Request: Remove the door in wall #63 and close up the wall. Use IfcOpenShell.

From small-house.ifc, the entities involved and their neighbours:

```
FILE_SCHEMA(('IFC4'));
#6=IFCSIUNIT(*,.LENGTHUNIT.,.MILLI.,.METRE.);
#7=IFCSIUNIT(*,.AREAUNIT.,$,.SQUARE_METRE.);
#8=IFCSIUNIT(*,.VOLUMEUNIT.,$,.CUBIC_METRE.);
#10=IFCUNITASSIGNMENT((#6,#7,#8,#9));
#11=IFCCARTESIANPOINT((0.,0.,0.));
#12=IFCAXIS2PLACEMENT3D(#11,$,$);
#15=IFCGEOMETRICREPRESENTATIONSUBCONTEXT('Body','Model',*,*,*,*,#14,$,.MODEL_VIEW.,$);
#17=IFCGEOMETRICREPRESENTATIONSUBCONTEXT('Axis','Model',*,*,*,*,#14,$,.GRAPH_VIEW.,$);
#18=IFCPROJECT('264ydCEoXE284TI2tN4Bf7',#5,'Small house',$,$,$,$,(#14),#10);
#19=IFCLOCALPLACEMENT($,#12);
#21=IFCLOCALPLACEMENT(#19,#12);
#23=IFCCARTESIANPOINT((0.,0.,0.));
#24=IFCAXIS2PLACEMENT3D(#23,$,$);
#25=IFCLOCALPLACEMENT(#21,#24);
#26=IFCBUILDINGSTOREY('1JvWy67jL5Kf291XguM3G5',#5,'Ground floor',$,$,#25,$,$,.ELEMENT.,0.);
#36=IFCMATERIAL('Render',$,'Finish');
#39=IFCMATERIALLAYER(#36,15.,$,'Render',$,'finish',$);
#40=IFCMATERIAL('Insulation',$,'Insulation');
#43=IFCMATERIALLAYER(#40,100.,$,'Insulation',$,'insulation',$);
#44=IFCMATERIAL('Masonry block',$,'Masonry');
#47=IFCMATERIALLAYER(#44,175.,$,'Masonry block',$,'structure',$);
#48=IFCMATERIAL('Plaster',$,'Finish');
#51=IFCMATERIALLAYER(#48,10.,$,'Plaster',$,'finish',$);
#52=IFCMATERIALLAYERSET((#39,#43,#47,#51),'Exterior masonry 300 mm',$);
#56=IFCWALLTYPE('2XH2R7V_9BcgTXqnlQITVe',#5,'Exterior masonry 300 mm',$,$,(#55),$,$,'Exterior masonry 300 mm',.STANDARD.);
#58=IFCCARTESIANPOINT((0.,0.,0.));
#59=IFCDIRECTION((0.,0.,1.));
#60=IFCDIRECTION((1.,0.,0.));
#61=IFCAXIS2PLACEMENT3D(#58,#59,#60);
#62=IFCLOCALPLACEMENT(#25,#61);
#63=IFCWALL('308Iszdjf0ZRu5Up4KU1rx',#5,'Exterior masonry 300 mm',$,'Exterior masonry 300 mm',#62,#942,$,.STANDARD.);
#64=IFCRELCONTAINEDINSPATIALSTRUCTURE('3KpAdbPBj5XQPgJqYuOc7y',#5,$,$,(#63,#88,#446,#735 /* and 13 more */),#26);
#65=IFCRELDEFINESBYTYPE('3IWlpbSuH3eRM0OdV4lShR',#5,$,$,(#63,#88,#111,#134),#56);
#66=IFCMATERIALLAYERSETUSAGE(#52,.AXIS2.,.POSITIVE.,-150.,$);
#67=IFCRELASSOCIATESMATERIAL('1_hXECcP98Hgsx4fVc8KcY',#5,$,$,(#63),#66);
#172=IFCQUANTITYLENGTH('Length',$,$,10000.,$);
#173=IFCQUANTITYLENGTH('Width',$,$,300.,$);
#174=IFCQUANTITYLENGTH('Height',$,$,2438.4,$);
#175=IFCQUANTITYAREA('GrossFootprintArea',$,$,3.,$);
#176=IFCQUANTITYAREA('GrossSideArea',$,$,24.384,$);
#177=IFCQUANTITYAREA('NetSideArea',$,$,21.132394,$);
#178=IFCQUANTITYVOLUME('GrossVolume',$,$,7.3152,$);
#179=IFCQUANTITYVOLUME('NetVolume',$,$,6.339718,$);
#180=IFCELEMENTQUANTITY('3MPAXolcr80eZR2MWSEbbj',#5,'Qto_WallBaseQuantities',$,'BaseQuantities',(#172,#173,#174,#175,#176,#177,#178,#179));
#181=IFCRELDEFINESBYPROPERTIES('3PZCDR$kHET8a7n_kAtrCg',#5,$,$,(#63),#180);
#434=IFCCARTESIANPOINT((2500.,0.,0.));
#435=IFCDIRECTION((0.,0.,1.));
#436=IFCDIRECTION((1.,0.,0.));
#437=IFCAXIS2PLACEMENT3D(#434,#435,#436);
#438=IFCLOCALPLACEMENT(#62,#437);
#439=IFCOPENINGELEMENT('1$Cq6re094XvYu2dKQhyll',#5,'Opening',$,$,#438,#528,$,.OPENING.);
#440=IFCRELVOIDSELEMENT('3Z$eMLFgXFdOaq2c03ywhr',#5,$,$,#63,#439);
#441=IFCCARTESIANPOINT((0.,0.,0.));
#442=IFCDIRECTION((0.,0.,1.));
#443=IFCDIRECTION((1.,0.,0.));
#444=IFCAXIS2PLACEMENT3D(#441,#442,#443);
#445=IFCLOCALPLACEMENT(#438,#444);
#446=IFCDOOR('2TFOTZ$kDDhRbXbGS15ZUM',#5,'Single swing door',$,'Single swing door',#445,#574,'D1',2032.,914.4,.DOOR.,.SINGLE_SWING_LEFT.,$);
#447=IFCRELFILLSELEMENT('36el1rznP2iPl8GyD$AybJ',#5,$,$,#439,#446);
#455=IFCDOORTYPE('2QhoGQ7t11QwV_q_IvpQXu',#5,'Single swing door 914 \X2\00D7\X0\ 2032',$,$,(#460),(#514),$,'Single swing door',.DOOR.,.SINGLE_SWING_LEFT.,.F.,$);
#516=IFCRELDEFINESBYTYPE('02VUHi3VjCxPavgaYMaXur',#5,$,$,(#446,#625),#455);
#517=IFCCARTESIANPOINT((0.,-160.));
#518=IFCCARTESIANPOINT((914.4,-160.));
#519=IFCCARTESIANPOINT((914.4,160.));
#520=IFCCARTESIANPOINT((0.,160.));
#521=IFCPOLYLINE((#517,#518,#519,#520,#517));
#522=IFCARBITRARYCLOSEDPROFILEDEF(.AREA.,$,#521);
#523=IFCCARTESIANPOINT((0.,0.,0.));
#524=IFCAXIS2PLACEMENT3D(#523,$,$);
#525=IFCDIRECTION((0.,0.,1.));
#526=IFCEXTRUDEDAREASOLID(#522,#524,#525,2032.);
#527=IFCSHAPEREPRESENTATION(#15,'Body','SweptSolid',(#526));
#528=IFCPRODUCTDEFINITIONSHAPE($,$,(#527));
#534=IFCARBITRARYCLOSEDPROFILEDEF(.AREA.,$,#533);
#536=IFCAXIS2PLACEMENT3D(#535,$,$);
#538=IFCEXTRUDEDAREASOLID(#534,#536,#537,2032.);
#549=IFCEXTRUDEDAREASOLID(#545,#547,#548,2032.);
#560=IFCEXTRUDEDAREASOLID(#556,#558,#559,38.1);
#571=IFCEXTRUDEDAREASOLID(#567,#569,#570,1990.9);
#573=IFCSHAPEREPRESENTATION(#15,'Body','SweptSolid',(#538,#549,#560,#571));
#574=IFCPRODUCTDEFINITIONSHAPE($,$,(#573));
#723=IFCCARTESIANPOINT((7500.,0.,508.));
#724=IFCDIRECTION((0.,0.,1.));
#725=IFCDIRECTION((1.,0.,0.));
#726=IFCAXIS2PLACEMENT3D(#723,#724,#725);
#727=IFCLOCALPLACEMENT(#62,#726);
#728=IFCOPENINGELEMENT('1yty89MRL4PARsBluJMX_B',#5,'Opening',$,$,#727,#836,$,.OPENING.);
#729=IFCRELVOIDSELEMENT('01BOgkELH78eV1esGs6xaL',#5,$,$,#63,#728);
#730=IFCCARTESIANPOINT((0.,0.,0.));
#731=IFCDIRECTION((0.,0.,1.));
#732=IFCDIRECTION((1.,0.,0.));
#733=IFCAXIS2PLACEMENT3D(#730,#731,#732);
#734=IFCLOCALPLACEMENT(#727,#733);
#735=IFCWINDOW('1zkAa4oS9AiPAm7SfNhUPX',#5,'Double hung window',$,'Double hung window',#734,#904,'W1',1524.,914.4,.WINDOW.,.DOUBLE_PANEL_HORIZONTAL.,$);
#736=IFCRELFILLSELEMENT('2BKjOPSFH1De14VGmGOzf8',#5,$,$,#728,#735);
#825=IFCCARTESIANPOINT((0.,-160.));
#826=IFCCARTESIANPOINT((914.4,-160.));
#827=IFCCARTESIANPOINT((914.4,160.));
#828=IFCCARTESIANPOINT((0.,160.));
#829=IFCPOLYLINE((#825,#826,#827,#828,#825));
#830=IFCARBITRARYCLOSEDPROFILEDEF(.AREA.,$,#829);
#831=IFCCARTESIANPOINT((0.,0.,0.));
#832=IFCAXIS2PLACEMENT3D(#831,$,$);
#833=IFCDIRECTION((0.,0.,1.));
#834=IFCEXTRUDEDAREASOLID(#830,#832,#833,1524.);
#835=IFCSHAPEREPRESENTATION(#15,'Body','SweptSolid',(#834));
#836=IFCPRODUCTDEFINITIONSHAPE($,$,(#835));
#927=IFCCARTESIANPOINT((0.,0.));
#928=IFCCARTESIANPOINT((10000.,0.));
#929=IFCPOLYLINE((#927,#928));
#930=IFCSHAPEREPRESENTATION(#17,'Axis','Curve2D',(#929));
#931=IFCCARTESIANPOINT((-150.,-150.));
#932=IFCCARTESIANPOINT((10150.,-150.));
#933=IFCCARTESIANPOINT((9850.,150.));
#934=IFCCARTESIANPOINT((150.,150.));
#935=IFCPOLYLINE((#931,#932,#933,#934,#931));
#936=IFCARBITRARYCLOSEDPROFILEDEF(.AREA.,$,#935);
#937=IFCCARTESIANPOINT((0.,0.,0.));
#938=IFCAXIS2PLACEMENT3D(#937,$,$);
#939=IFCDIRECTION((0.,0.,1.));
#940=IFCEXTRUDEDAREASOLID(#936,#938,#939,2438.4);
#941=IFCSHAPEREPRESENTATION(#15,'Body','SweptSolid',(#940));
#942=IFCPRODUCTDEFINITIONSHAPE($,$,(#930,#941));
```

```python
import ifcopenshell
import ifcopenshell.api.feature
import ifcopenshell.api.pset
import ifcopenshell.api.root
import ifcopenshell.geom
import ifcopenshell.util.element
import ifcopenshell.util.shape
import ifcopenshell.util.unit

model = ifcopenshell.open("small-house.ifc")
area_scale = ifcopenshell.util.unit.calculate_unit_scale(model, "AREAUNIT")
volume_scale = ifcopenshell.util.unit.calculate_unit_scale(model, "VOLUMEUNIT")
settings = ifcopenshell.geom.settings()


def volume(element):
    """Net volume in cubic metres, openings subtracted."""
    shape = ifcopenshell.geom.create_shape(settings, element)
    return ifcopenshell.util.shape.get_volume(shape.geometry)


door = model.by_guid("2TFOTZ$kDDhRbXbGS15ZUM")
opening = door.FillsVoids[0].RelatingOpeningElement
wall = opening.VoidsElements[0].RelatingBuildingElement
before = volume(wall)

ifcopenshell.api.root.remove_product(model, product=door)
ifcopenshell.api.feature.remove_feature(model, feature=opening)

after = volume(wall)
thickness = 0.3  # wall thickness in metres

# Update the wall's stored quantities.
qto = model.by_id(ifcopenshell.util.element.get_pset(wall, "Qto_WallBaseQuantities", should_inherit=False)["id"])
ifcopenshell.api.pset.edit_qto(model, qto=qto, properties={
    "NetSideArea": after / thickness / area_scale,
    "NetVolume": after / volume_scale,
})

print(f"wall volume {before:.3f} -> {after:.3f} m3")

model.write("small-house_updated.ifc")
```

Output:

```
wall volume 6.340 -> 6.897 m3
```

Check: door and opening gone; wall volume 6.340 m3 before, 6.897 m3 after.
